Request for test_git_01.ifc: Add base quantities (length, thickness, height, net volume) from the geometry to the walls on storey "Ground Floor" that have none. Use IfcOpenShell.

First a look at what the model holds.

```python
import ifcopenshell
import ifcopenshell.util.element
import ifcopenshell.util.unit

model = ifcopenshell.open("test_git_01.ifc")
print(model.schema)
for unit_type in ("LENGTHUNIT", "AREAUNIT", "VOLUMEUNIT"):
    print(unit_type, ifcopenshell.util.unit.calculate_unit_scale(model, unit_type))
storey = next(s for s in model.by_type("IfcBuildingStorey") if s.Name == "Ground Floor")
walls = [e for e in ifcopenshell.util.element.get_decomposition(storey) if e.is_a("IfcWall")]
for e in sorted(walls, key=lambda e: e.id()):
    print(e.id(), e.is_a(), e.Name, list(ifcopenshell.util.element.get_psets(e, qtos_only=True)), sep=" | ")
```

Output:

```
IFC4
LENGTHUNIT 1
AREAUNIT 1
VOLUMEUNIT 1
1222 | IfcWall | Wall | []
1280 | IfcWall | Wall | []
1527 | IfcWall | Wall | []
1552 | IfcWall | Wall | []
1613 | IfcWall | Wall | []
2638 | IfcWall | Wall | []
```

```python
import ifcopenshell
import ifcopenshell.api.pset
import ifcopenshell.geom
import ifcopenshell.util.element
import ifcopenshell.util.shape
import ifcopenshell.util.unit

model = ifcopenshell.open("test_git_01.ifc")
unit_scale = ifcopenshell.util.unit.calculate_unit_scale(model)
volume_scale = ifcopenshell.util.unit.calculate_unit_scale(model, "VOLUMEUNIT")
settings = ifcopenshell.geom.settings()

storey = next(s for s in model.by_type("IfcBuildingStorey") if s.Name == "Ground Floor")
walls = [e for e in ifcopenshell.util.element.get_decomposition(storey) if e.is_a("IfcWall")]

for e in sorted(walls, key=lambda e: e.id()):
    if ifcopenshell.util.element.get_psets(e, qtos_only=True, should_inherit=False):
        continue
    # Geometry comes back in metres, in the element's own axes.
    shape = ifcopenshell.geom.create_shape(settings, e)
    values = {
        "Length": ifcopenshell.util.shape.get_x(shape.geometry) / unit_scale,
        "Width": ifcopenshell.util.shape.get_y(shape.geometry) / unit_scale,
        "Height": ifcopenshell.util.shape.get_z(shape.geometry) / unit_scale,
        "NetVolume": ifcopenshell.util.shape.get_volume(shape.geometry) / volume_scale,
    }
    qto = ifcopenshell.api.pset.add_qto(model, product=e, name="Qto_WallBaseQuantities")
    ifcopenshell.api.pset.edit_qto(model, qto=qto, properties=values)
    print(e.id(), {k: round(v, 3) for k, v in values.items()})

model.write("test_git_01_rev.ifc")
```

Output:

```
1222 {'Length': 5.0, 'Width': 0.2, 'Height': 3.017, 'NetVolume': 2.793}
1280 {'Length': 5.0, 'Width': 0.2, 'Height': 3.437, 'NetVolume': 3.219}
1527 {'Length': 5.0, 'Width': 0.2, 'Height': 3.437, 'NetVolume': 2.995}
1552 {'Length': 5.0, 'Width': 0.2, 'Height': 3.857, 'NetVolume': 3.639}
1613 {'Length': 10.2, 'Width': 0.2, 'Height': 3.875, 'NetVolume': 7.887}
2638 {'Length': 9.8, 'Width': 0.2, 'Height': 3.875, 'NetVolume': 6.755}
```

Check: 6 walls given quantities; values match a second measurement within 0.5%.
